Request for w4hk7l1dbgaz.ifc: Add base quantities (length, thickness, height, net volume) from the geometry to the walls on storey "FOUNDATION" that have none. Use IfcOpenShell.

First a look at what the model holds.

```python
import ifcopenshell
import ifcopenshell.util.element
import ifcopenshell.util.unit

model = ifcopenshell.open("w4hk7l1dbgaz.ifc")
print(model.schema)
for unit_type in ("LENGTHUNIT", "AREAUNIT", "VOLUMEUNIT"):
    print(unit_type, ifcopenshell.util.unit.calculate_unit_scale(model, unit_type))
storey = next(s for s in model.by_type("IfcBuildingStorey") if s.Name == "FOUNDATION")
walls = [e for e in ifcopenshell.util.element.get_decomposition(storey) if e.is_a("IfcWall")]
for e in sorted(walls, key=lambda e: e.id()):
    print(e.id(), e.is_a(), e.Name, list(ifcopenshell.util.element.get_psets(e, qtos_only=True)), sep=" | ")
```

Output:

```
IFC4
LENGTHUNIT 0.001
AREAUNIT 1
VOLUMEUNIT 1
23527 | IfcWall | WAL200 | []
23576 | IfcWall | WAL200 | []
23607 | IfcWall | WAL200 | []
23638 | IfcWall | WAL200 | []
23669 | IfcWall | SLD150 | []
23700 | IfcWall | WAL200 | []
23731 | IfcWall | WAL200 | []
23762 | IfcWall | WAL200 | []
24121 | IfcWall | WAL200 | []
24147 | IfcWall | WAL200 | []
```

```python
import ifcopenshell
import ifcopenshell.api.pset
import ifcopenshell.geom
import ifcopenshell.util.element
import ifcopenshell.util.shape
import ifcopenshell.util.unit

model = ifcopenshell.open("w4hk7l1dbgaz.ifc")
unit_scale = ifcopenshell.util.unit.calculate_unit_scale(model)
volume_scale = ifcopenshell.util.unit.calculate_unit_scale(model, "VOLUMEUNIT")
settings = ifcopenshell.geom.settings()

storey = next(s for s in model.by_type("IfcBuildingStorey") if s.Name == "FOUNDATION")
walls = [e for e in ifcopenshell.util.element.get_decomposition(storey) if e.is_a("IfcWall")]

for e in sorted(walls, key=lambda e: e.id()):
    if ifcopenshell.util.element.get_psets(e, qtos_only=True, should_inherit=False):
        continue
    # Geometry comes back in metres, in the element's own axes.
    shape = ifcopenshell.geom.create_shape(settings, e)
    values = {
        "Length": ifcopenshell.util.shape.get_x(shape.geometry) / unit_scale,
        "Width": ifcopenshell.util.shape.get_y(shape.geometry) / unit_scale,
        "Height": ifcopenshell.util.shape.get_z(shape.geometry) / unit_scale,
        "NetVolume": ifcopenshell.util.shape.get_volume(shape.geometry) / volume_scale,
    }
    qto = ifcopenshell.api.pset.add_qto(model, product=e, name="Qto_WallBaseQuantities")
    ifcopenshell.api.pset.edit_qto(model, qto=qto, properties=values)
    print(e.id(), {k: round(v, 3) for k, v in values.items()})

model.write("w4hk7l1dbgaz_edited.ifc")
```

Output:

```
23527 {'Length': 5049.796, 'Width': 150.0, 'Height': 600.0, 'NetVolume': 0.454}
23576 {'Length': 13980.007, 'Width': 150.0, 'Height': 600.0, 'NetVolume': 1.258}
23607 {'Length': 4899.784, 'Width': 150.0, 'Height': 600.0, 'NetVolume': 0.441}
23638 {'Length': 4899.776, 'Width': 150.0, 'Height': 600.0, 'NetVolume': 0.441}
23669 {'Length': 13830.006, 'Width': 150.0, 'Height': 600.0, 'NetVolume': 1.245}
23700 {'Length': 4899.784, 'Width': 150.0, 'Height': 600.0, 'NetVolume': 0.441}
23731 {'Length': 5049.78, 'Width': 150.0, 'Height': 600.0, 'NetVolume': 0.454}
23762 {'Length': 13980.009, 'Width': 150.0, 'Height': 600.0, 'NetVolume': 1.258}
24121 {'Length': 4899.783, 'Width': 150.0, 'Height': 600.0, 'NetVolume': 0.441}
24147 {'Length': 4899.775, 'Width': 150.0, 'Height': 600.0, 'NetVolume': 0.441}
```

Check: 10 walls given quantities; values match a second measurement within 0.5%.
